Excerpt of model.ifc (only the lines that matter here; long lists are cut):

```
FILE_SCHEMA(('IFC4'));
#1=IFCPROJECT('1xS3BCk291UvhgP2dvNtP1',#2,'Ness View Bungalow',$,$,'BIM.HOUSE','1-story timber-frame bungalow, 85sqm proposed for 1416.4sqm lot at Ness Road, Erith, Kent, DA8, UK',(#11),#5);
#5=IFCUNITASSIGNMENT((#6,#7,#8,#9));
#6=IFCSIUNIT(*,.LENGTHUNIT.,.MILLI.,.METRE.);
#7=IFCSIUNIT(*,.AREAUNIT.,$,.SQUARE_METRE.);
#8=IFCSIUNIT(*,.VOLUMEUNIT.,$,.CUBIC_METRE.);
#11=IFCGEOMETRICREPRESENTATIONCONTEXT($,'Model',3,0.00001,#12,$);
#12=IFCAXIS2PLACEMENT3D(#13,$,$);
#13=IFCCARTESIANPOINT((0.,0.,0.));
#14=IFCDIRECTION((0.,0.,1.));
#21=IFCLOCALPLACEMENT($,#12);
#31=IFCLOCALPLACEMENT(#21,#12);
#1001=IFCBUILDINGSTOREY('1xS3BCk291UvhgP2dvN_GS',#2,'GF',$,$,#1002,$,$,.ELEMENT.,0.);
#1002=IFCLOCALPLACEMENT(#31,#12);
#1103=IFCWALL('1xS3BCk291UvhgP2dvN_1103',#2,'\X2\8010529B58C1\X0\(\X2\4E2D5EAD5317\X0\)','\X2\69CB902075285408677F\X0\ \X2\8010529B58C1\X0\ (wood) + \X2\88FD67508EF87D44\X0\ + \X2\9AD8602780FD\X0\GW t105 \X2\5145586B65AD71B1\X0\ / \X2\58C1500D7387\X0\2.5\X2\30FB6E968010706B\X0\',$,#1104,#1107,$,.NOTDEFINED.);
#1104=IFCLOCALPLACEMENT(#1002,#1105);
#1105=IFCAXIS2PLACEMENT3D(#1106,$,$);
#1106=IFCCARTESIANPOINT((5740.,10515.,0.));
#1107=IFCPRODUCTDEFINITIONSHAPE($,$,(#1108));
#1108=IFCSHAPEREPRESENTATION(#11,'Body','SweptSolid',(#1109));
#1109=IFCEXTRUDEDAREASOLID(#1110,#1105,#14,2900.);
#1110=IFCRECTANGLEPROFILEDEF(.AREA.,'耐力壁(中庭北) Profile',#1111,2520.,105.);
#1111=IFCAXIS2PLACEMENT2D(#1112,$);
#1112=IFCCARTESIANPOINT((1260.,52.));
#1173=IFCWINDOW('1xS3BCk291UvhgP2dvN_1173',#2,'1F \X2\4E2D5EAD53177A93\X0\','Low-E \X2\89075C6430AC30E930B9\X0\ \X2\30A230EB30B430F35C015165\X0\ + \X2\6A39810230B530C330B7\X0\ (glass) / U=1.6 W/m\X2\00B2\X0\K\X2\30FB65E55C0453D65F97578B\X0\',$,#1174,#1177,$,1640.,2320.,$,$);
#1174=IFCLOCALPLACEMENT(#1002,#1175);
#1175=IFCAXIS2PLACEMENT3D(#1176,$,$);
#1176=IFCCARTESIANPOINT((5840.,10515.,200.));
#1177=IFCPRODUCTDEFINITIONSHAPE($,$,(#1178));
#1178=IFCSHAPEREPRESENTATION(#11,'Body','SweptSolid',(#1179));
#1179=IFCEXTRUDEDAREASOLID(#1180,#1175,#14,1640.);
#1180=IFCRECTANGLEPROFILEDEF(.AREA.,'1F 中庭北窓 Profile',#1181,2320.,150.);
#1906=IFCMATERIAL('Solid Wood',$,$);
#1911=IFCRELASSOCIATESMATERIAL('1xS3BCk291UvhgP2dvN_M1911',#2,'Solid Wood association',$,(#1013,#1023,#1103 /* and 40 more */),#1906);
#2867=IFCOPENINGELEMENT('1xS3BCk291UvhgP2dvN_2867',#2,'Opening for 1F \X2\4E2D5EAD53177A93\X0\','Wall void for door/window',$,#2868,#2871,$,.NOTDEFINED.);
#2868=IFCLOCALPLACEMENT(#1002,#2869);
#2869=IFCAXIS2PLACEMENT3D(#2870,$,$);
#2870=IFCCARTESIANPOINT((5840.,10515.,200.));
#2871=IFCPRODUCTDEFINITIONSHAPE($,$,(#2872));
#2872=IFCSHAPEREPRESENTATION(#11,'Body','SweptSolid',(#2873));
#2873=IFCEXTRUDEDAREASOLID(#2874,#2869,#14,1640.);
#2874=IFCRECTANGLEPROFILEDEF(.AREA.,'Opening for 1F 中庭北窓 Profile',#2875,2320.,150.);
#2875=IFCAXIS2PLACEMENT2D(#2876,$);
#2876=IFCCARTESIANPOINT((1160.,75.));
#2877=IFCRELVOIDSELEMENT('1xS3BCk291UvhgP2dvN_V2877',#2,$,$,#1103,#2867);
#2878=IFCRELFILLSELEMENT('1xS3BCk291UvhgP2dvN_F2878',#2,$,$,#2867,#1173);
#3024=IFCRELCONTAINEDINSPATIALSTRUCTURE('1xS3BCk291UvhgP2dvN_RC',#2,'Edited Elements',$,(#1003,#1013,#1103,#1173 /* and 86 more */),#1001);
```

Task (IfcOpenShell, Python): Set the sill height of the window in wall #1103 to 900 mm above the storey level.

```python
import numpy as np
import ifcopenshell
import ifcopenshell.api.geometry
import ifcopenshell.geom
import ifcopenshell.util.element
import ifcopenshell.util.placement
import ifcopenshell.util.shape
import ifcopenshell.util.unit

model = ifcopenshell.open("model.ifc")
unit_scale = ifcopenshell.util.unit.calculate_unit_scale(model)

window = model.by_guid("1xS3BCk291UvhgP2dvN_1173")
opening = window.FillsVoids[0].RelatingOpeningElement
storey = ifcopenshell.util.element.get_container(window, ifc_class="IfcBuildingStorey")
level = ifcopenshell.util.placement.get_local_placement(storey.ObjectPlacement)[2, 3]

# The opening's origin need not be at the sill, so measure its lowest point.
shape = ifcopenshell.geom.create_shape(ifcopenshell.geom.settings(), opening)
bottom = ifcopenshell.util.shape.get_shape_bottom_elevation(shape, shape.geometry) / unit_scale
dz = level + 0.9 / unit_scale - bottom

shift = np.array([0.0, 0.0, dz])
# The window is not placed relative to its opening, so move both.
for product in (opening, window):
    matrix = ifcopenshell.util.placement.get_local_placement(product.ObjectPlacement)
    matrix[:3, 3] += shift
    ifcopenshell.api.geometry.edit_object_placement(model, product=product, matrix=matrix, is_si=False)

print(f"moved by {dz * unit_scale:+.3f} m")

model.write("model-out.ifc")
```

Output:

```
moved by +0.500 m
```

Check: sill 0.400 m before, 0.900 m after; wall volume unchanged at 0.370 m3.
